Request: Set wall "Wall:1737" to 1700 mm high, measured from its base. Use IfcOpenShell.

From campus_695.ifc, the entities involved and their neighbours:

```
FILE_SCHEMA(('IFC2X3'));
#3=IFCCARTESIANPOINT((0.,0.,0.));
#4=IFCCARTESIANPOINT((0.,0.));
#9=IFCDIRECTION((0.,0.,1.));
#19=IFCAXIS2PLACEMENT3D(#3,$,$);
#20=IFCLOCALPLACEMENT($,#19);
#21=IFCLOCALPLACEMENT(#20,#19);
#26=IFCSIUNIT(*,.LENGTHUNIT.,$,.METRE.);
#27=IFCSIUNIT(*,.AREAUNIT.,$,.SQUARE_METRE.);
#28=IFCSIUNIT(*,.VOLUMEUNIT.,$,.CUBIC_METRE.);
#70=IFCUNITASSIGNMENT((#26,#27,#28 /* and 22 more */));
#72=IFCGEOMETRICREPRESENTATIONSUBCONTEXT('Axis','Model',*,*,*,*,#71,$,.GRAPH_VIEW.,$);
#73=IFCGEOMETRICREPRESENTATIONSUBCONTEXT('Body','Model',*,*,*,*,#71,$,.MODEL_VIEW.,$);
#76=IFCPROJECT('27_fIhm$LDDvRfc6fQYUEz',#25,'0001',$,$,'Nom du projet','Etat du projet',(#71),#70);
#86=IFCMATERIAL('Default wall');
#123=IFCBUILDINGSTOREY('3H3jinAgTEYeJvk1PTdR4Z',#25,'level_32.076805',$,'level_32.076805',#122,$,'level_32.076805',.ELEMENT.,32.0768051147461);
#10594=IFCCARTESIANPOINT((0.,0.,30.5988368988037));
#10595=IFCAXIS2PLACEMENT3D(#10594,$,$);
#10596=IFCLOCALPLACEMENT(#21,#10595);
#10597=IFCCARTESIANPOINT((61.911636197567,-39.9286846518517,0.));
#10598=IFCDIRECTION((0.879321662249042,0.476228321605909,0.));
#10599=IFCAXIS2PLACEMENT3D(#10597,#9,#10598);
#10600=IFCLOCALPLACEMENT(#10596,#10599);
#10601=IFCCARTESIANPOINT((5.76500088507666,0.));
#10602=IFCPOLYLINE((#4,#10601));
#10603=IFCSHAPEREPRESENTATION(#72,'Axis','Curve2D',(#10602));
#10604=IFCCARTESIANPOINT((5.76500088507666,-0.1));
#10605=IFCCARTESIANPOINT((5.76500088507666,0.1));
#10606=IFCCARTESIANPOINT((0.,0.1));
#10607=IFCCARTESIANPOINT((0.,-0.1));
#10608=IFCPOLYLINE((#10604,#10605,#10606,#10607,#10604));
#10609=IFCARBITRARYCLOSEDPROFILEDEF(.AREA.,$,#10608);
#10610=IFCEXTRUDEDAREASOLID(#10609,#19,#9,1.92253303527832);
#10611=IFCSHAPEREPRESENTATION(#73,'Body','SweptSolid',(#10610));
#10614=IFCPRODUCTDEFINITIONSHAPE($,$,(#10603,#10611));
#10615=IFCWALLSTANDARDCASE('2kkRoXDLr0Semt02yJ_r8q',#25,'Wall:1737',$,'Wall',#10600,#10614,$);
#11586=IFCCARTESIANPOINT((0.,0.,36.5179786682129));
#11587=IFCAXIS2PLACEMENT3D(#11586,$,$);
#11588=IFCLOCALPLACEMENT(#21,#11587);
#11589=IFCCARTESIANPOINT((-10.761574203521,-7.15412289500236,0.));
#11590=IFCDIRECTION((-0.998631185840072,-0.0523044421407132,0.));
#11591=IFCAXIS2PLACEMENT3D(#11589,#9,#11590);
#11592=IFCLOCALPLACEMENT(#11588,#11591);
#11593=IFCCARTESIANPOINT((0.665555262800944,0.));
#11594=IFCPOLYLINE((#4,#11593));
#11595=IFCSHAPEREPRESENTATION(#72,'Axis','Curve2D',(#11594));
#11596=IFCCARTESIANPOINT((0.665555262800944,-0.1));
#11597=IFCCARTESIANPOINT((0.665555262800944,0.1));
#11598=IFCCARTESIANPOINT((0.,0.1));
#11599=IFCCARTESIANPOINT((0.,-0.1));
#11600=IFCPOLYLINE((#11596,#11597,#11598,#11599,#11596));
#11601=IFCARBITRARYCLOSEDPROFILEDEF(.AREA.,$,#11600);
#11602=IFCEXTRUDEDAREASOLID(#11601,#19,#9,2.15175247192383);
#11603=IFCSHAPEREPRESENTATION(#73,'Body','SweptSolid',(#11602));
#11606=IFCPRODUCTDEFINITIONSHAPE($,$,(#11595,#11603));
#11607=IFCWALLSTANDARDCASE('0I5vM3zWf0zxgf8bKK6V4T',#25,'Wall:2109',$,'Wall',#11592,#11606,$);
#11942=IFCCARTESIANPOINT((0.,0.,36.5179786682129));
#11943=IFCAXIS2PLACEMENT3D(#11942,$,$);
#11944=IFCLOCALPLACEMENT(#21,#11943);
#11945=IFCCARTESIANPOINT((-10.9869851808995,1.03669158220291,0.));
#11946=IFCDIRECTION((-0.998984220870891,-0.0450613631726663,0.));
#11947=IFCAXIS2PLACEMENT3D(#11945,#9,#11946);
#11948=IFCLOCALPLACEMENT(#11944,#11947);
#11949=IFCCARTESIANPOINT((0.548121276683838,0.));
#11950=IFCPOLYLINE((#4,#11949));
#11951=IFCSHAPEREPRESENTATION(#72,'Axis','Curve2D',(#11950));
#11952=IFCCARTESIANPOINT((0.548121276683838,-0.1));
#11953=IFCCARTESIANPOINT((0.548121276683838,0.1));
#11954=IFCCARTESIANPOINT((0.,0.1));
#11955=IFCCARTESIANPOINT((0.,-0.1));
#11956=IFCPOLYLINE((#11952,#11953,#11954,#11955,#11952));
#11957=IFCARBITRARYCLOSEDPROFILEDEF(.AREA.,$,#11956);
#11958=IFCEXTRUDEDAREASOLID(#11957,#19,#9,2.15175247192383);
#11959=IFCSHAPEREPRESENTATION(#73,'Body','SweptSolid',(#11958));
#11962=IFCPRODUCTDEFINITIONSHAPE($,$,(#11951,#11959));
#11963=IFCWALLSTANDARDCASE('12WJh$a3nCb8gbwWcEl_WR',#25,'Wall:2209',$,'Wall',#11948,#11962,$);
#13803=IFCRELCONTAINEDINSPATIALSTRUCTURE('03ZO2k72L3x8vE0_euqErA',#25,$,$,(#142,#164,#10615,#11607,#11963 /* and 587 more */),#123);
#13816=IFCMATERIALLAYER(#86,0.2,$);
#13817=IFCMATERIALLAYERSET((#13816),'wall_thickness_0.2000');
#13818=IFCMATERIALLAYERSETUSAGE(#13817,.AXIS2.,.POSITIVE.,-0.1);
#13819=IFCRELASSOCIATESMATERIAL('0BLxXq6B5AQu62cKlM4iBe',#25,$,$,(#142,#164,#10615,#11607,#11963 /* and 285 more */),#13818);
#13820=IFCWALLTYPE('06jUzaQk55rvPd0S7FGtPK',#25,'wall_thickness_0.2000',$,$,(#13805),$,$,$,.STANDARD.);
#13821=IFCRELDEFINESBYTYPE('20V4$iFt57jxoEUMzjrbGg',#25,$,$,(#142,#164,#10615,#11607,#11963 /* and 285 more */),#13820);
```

```python
import ifcopenshell
import ifcopenshell.geom
import ifcopenshell.util.representation
import ifcopenshell.util.shape
import ifcopenshell.util.unit

model = ifcopenshell.open("campus_695.ifc")
unit_scale = ifcopenshell.util.unit.calculate_unit_scale(model)
settings = ifcopenshell.geom.settings()


def volume(element):
    """Net volume in cubic metres, openings subtracted."""
    shape = ifcopenshell.geom.create_shape(settings, element)
    return ifcopenshell.util.shape.get_volume(shape.geometry)


wall = model.by_guid("2kkRoXDLr0Semt02yJ_r8q")
before = volume(wall)

body = ifcopenshell.util.representation.get_representation(wall, "Model", "Body")
solid = body.Items[0]
old_height = solid.Depth
solid.Depth = 1.7 / unit_scale
after = volume(wall)

print(f"height {old_height:g} -> {solid.Depth:g}, volume {before:.3f} -> {after:.3f} m3")

model.write("campus_695-out.ifc")
```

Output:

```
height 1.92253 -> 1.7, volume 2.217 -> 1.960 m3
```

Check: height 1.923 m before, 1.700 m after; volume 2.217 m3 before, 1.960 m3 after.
